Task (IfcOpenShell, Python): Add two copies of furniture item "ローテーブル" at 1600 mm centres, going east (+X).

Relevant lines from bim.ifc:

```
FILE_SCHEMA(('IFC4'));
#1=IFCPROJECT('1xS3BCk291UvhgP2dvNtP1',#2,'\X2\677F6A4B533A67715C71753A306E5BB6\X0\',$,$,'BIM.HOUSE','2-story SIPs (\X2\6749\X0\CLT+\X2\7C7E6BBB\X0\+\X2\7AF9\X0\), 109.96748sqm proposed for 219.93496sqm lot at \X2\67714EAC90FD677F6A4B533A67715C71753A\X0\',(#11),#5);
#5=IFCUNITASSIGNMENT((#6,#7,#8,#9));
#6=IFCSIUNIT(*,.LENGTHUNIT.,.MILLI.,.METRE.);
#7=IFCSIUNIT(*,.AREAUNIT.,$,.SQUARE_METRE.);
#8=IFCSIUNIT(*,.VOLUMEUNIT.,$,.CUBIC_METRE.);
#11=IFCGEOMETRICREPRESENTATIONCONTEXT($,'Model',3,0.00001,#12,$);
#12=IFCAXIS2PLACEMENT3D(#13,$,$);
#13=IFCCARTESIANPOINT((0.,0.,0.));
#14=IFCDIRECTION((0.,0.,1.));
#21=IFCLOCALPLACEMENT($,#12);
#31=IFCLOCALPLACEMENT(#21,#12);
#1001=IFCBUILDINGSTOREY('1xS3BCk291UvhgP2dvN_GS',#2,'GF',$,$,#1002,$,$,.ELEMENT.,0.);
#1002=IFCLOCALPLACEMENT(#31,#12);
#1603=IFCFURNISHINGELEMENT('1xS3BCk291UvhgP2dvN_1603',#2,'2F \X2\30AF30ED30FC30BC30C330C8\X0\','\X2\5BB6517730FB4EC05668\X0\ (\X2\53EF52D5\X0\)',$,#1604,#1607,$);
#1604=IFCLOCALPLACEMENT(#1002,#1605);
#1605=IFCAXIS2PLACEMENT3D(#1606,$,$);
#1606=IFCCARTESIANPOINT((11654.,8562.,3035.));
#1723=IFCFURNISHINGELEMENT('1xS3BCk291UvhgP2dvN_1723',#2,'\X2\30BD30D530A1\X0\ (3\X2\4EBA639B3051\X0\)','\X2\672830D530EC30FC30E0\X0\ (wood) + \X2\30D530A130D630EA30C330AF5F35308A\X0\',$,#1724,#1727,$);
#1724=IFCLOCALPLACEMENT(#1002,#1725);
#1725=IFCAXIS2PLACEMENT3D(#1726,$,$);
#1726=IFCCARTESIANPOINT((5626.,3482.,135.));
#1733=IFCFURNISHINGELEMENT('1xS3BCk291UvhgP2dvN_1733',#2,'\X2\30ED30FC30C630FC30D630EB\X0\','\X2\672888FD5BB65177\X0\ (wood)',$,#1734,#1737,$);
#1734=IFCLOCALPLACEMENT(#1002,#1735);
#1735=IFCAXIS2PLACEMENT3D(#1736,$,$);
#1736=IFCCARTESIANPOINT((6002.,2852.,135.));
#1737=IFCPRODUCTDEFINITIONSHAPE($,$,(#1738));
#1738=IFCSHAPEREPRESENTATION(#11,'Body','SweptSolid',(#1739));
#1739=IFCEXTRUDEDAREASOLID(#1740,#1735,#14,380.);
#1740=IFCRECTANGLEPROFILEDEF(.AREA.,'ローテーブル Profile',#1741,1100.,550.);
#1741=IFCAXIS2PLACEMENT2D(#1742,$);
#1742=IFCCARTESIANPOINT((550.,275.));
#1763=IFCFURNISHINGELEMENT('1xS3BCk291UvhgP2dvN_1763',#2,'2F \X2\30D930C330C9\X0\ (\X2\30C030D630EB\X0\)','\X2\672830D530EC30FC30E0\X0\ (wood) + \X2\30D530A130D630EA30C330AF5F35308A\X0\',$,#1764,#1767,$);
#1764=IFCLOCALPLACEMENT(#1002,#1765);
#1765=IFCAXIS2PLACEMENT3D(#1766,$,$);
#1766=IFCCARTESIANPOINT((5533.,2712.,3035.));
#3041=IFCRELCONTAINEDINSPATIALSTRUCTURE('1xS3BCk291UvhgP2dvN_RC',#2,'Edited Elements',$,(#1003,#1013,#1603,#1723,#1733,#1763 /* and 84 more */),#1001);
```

```python
import numpy as np
import ifcopenshell
import ifcopenshell.api.geometry
import ifcopenshell.api.root
import ifcopenshell.util.element
import ifcopenshell.util.placement

model = ifcopenshell.open("bim.ifc")


def reuse_history(source, copy):
    """copy_class also copies each property set's owner history, people and application; keep the originals."""
    for rel in copy.IsDefinedBy:
        if rel.is_a("IfcRelDefinesByProperties") and (history := rel.RelatingPropertyDefinition.OwnerHistory):
            rel.RelatingPropertyDefinition.OwnerHistory = source.OwnerHistory
            ifcopenshell.util.element.remove_deep2(model, history)


source = model.by_guid("1xS3BCk291UvhgP2dvN_1733")
base = ifcopenshell.util.placement.get_local_placement(source.ObjectPlacement)
step = np.array([1.0, 0.0, 0.0]) * 1600.0

for i in range(1, 3):
    copy = ifcopenshell.api.root.copy_class(model, product=source)
    copy.Representation = ifcopenshell.util.element.copy_deep(
        model, source.Representation, exclude=["IfcGeometricRepresentationContext", "IfcRepresentationMap"]
    )
    reuse_history(source, copy)
    matrix = base.copy()
    matrix[:3, 3] += i * step
    print("added at", matrix[:3, 3].round(3) + 0.0)
    ifcopenshell.api.geometry.edit_object_placement(model, product=copy, matrix=matrix, is_si=False)

model.write("bim_v2.ifc")
```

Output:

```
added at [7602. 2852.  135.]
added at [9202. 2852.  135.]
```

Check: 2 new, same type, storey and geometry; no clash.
